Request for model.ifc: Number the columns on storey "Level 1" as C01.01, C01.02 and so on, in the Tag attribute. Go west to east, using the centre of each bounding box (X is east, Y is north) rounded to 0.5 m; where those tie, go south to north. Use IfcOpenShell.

First a look at what the model holds.

```python
import ifcopenshell
import ifcopenshell.util.element
import ifcopenshell.util.placement

model = ifcopenshell.open("model.ifc")
print(model.schema)
storey = next(s for s in model.by_type("IfcBuildingStorey") if s.Name == "Level 1")
columns = [e for e in ifcopenshell.util.element.get_decomposition(storey) if e.is_a("IfcColumn")]
for e in sorted(columns, key=lambda e: e.id()):
    origin = ifcopenshell.util.placement.get_local_placement(e.ObjectPlacement)[:3, 3]
    print(e.id(), e.Tag, e.Name, origin.round(2) + 0.0, sep=" | ")
```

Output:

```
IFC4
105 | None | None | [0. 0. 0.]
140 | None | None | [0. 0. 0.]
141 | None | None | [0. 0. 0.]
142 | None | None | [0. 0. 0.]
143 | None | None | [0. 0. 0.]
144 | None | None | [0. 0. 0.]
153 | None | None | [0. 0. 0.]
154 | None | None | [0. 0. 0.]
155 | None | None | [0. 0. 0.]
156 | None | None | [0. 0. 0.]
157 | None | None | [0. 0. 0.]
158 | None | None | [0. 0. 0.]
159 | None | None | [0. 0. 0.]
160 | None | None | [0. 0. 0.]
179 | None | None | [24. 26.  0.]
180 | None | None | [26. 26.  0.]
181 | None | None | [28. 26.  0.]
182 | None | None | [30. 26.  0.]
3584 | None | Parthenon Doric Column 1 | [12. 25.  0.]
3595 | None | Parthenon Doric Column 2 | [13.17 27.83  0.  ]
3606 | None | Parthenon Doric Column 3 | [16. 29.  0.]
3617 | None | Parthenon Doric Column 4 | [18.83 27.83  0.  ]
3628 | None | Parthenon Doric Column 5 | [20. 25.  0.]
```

```python
import ifcopenshell
import ifcopenshell.geom
import ifcopenshell.util.element
import ifcopenshell.util.shape

model = ifcopenshell.open("model.ifc")
settings = ifcopenshell.geom.settings()
settings.set("use-world-coords", True)


def centre(element):
    shape = ifcopenshell.geom.create_shape(settings, element)
    return ifcopenshell.util.shape.get_bbox_centroid(shape.geometry)


storey = next(s for s in model.by_type("IfcBuildingStorey") if s.Name == "Level 1")
columns = [e for e in ifcopenshell.util.element.get_decomposition(storey) if e.is_a("IfcColumn")]

# Insertion points can sit at a corner or the storey origin, so sort by the geometry (in metres).
centres = {e: centre(e) for e in columns}
columns.sort(key=lambda e: (round(centres[e][0] / 0.5), centres[e][1]))

for i, e in enumerate(columns, start=1):
    number = f"C01.{i:02d}"
    e.Tag = number
    print(e.id(), number)

model.write("model_rev.ifc")
```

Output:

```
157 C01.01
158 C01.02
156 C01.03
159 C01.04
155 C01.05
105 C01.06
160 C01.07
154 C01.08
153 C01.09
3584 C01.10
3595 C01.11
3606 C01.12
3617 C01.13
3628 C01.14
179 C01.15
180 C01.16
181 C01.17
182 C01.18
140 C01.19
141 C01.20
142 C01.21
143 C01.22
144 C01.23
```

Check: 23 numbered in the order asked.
